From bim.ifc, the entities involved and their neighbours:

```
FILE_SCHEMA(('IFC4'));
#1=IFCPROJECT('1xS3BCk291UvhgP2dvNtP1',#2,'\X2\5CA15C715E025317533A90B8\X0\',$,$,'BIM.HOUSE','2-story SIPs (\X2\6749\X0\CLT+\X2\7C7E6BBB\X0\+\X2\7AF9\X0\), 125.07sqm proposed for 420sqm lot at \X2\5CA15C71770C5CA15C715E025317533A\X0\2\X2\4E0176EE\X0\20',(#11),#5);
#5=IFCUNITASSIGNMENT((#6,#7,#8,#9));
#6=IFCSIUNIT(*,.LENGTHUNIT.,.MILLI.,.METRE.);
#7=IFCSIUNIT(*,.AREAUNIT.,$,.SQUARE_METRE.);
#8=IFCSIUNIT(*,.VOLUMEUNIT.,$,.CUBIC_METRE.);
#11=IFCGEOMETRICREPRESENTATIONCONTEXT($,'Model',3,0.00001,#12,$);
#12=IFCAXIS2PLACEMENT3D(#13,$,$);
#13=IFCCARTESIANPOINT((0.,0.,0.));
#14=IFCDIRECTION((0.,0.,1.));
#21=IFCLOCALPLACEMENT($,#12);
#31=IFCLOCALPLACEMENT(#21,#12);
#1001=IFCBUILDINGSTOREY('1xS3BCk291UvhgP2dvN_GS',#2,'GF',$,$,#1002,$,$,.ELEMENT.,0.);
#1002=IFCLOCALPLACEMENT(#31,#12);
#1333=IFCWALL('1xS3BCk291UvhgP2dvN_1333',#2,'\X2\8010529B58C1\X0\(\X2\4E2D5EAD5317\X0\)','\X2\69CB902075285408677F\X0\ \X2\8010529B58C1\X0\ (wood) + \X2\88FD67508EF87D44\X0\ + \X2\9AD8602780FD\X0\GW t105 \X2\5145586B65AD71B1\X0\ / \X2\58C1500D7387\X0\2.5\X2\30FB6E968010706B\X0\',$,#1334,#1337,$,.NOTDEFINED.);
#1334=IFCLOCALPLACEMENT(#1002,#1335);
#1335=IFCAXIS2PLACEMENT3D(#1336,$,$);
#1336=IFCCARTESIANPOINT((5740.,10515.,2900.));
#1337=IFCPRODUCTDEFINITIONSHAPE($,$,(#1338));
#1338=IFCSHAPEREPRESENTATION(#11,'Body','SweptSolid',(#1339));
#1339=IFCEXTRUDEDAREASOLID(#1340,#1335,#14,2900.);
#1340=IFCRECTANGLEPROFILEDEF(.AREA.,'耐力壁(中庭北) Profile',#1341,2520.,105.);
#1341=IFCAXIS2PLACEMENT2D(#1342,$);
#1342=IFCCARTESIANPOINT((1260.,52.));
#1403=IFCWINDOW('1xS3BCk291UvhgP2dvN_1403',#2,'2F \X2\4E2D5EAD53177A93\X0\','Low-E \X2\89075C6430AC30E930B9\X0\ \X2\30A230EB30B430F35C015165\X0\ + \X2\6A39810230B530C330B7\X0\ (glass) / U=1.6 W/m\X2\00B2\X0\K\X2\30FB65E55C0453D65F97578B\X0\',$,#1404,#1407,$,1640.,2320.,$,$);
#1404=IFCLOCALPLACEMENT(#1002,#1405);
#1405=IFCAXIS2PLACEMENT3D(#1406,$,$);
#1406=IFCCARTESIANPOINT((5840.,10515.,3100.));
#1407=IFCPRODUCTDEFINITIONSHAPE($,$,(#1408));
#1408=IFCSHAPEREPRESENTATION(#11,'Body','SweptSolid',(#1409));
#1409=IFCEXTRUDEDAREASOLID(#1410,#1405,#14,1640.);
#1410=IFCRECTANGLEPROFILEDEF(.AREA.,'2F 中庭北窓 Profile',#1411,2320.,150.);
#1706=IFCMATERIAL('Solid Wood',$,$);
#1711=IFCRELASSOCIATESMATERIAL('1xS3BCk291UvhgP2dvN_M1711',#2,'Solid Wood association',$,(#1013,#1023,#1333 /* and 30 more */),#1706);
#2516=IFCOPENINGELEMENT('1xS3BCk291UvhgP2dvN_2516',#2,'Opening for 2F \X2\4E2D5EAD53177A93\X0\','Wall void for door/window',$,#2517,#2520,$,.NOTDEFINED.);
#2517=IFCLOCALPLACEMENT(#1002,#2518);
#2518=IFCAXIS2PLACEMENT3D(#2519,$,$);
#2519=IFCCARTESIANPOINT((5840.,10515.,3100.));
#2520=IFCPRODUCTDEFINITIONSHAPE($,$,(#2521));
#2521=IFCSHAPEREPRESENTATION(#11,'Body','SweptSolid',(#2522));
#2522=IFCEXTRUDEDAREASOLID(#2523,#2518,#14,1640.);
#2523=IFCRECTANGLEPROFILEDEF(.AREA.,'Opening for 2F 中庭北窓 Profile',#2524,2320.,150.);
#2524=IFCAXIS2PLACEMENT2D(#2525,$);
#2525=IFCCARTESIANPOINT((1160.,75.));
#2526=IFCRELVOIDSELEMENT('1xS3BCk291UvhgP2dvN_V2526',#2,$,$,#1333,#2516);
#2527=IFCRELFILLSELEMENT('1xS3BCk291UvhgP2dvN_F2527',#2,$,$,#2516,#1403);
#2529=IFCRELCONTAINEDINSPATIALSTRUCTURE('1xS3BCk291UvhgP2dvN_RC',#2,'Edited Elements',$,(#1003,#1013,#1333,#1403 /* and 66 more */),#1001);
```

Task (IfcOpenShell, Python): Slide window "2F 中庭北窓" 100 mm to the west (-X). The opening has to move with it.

```python
import ifcopenshell
import ifcopenshell.api.geometry
import ifcopenshell.util.placement
import ifcopenshell.util.unit

model = ifcopenshell.open("bim.ifc")
unit_scale = ifcopenshell.util.unit.calculate_unit_scale(model)

window = model.by_guid("1xS3BCk291UvhgP2dvN_1403")
opening = window.FillsVoids[0].RelatingOpeningElement
wall = opening.VoidsElements[0].RelatingBuildingElement

wall_matrix = ifcopenshell.util.placement.get_local_placement(wall.ObjectPlacement)
shift = wall_matrix[:3, 0] * -0.1 / unit_scale
before = ifcopenshell.util.placement.get_local_placement(window.ObjectPlacement)[:3, 3].copy()

# The window is not placed relative to its opening, so move both.
for product in (opening, window):
    matrix = ifcopenshell.util.placement.get_local_placement(product.ObjectPlacement)
    matrix[:3, 3] += shift
    ifcopenshell.api.geometry.edit_object_placement(model, product=product, matrix=matrix, is_si=False)

after = ifcopenshell.util.placement.get_local_placement(window.ObjectPlacement)[:3, 3]
print("window moved by", (after - before).round(3) + 0.0)

model.write("bim_rev.ifc")
```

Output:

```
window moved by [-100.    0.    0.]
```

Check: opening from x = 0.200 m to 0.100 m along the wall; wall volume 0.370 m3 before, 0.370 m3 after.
